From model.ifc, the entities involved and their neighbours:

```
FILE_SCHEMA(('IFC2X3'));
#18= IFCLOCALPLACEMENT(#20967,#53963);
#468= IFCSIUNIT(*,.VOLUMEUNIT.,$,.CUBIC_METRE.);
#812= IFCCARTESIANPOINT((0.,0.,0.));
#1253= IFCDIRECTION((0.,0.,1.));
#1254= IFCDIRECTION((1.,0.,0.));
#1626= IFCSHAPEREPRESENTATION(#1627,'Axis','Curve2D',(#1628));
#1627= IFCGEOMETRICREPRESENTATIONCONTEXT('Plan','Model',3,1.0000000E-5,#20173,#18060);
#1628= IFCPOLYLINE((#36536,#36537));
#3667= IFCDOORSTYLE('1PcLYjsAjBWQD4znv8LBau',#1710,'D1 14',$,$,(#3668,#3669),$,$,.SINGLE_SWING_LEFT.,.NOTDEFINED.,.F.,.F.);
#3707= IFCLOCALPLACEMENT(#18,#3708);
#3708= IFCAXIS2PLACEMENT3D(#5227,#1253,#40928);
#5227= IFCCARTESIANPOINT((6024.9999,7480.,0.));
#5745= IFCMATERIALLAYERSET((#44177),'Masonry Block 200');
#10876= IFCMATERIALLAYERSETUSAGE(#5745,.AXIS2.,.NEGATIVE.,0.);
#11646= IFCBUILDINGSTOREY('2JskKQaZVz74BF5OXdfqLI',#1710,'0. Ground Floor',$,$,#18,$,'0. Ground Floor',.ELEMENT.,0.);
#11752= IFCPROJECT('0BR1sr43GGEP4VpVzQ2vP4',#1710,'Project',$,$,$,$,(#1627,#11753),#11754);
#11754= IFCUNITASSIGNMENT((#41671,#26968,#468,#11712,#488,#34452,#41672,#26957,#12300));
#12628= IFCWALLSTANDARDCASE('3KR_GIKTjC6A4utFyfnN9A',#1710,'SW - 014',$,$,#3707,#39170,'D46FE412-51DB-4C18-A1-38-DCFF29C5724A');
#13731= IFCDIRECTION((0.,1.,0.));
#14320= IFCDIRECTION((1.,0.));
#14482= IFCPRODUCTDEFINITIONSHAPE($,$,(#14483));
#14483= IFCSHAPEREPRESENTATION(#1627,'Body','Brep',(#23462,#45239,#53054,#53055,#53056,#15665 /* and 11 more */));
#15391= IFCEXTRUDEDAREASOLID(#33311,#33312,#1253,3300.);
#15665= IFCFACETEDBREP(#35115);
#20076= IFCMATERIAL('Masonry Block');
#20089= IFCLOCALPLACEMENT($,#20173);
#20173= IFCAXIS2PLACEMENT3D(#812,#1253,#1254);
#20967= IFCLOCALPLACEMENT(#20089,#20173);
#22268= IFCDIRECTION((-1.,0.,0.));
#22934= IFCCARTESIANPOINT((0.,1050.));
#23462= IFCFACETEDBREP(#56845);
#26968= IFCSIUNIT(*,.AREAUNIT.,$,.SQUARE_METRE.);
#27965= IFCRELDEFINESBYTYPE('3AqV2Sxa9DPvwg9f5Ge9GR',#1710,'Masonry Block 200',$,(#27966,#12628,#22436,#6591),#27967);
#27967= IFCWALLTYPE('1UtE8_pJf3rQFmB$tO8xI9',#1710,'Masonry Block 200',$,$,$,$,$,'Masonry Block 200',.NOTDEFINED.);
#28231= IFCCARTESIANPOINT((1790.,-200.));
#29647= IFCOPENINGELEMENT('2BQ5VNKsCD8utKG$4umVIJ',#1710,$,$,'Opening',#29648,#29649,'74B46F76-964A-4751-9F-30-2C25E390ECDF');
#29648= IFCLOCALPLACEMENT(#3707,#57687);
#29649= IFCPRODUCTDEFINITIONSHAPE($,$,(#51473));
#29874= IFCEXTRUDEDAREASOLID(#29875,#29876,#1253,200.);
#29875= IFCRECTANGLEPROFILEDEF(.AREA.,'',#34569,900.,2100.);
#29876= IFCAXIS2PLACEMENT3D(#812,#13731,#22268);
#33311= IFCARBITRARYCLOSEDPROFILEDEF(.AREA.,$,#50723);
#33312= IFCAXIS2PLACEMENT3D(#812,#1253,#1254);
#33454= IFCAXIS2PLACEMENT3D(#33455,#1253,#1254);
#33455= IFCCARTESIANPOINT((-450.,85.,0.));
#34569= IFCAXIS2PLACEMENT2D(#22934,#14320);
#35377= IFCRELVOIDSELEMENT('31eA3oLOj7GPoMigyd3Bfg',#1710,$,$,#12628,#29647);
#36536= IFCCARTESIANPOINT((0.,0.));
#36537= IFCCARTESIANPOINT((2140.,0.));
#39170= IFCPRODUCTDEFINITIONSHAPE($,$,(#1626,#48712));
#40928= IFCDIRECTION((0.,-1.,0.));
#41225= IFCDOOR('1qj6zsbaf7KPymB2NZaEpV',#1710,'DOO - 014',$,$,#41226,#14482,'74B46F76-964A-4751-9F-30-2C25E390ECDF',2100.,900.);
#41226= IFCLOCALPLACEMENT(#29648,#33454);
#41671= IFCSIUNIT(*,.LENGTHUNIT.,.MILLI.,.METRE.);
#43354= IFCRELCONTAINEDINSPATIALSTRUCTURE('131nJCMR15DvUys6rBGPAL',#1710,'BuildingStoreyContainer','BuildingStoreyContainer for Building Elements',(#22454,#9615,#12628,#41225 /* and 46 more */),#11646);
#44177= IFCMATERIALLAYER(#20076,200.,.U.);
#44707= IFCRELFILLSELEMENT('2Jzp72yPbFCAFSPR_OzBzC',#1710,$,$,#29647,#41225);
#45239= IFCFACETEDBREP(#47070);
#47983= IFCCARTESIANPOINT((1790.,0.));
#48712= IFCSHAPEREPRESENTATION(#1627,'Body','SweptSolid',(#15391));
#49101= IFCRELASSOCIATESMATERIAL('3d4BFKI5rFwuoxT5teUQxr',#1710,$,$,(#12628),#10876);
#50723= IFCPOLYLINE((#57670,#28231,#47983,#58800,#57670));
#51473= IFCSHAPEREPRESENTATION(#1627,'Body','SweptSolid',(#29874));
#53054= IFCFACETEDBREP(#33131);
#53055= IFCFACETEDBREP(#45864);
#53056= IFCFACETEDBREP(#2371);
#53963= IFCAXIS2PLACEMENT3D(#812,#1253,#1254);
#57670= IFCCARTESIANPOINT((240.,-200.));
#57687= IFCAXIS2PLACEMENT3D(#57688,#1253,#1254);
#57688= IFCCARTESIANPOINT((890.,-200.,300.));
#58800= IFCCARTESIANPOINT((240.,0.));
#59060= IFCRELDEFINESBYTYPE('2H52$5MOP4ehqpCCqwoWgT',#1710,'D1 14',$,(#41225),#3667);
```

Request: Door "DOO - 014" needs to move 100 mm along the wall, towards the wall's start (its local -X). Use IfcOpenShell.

```python
import ifcopenshell
import ifcopenshell.api.geometry
import ifcopenshell.util.placement
import ifcopenshell.util.unit

model = ifcopenshell.open("model.ifc")
unit_scale = ifcopenshell.util.unit.calculate_unit_scale(model)

door = model.by_id(41225)
opening = door.FillsVoids[0].RelatingOpeningElement
wall = opening.VoidsElements[0].RelatingBuildingElement

wall_matrix = ifcopenshell.util.placement.get_local_placement(wall.ObjectPlacement)
shift = wall_matrix[:3, 0] * -0.1 / unit_scale
before = ifcopenshell.util.placement.get_local_placement(door.ObjectPlacement)[:3, 3].copy()

# The door is placed relative to its opening, so it follows when the opening moves.
matrix = ifcopenshell.util.placement.get_local_placement(opening.ObjectPlacement)
matrix[:3, 3] += shift
ifcopenshell.api.geometry.edit_object_placement(
    model, product=opening, matrix=matrix, is_si=False, should_transform_children=True
)

after = ifcopenshell.util.placement.get_local_placement(door.ObjectPlacement)[:3, 3]
print("door moved by", (after - before).round(3) + 0.0)

model.write("model-out.ifc")
```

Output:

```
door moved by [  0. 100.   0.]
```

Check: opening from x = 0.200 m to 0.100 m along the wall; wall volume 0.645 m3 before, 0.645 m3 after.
